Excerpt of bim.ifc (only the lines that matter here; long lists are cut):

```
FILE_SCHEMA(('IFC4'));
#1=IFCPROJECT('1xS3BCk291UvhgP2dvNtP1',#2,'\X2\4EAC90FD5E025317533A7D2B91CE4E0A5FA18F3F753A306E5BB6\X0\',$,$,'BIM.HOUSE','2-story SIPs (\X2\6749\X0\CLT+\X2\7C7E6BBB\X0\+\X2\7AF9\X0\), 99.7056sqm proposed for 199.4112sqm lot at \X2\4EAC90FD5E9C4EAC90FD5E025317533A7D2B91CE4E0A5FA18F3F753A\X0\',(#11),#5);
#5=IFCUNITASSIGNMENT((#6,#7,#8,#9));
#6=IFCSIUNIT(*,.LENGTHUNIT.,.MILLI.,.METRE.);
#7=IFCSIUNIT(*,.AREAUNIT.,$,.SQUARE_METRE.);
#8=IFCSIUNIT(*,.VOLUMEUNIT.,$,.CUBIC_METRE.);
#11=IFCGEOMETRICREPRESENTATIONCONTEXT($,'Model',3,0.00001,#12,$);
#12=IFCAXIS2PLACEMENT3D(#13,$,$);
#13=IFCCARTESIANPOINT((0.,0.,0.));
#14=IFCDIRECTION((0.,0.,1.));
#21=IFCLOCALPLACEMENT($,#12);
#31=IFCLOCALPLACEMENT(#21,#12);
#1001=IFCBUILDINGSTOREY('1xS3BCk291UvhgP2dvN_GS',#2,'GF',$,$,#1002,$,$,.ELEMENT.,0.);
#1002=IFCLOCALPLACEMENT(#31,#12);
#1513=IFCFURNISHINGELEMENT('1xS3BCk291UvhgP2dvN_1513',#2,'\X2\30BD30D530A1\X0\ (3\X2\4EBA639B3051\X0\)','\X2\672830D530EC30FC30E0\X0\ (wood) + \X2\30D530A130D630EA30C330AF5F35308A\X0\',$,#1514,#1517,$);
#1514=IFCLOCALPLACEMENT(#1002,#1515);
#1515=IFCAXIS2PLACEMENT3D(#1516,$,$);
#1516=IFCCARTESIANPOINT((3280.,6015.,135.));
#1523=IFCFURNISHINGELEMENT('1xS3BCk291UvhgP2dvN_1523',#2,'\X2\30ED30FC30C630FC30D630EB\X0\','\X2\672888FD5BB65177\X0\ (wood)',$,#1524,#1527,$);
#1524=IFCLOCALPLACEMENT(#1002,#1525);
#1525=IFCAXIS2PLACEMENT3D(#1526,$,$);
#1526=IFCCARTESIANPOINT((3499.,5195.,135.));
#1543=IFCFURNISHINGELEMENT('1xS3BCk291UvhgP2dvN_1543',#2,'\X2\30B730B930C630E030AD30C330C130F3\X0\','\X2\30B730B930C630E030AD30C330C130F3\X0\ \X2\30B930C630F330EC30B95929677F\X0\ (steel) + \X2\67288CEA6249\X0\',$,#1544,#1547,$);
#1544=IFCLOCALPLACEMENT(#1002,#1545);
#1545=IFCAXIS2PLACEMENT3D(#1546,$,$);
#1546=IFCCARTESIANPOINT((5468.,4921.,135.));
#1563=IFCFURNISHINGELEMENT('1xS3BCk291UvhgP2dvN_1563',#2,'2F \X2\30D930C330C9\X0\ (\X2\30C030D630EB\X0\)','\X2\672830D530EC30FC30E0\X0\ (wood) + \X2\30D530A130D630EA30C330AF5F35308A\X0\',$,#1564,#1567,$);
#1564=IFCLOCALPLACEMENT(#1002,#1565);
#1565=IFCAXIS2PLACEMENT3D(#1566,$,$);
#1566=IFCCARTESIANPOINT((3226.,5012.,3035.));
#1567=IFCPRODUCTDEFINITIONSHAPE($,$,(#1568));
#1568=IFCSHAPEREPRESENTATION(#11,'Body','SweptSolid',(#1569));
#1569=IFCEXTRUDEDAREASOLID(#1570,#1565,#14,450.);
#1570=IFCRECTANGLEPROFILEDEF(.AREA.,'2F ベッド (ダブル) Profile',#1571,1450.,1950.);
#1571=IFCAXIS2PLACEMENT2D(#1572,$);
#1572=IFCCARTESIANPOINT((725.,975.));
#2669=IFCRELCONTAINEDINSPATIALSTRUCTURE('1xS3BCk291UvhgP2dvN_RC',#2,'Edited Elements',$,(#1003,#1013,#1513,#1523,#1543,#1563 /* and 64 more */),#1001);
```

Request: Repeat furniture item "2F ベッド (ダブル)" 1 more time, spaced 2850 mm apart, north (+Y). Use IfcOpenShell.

```python
import numpy as np
import ifcopenshell
import ifcopenshell.api.geometry
import ifcopenshell.api.root
import ifcopenshell.util.element
import ifcopenshell.util.placement
import ifcopenshell.util.unit

model = ifcopenshell.open("bim.ifc")
unit_scale = ifcopenshell.util.unit.calculate_unit_scale(model)


def reuse_history(source, copy):
    """copy_class also copies each property set's owner history, people and application; keep the originals."""
    for rel in copy.IsDefinedBy:
        if rel.is_a("IfcRelDefinesByProperties") and (history := rel.RelatingPropertyDefinition.OwnerHistory):
            rel.RelatingPropertyDefinition.OwnerHistory = source.OwnerHistory
            ifcopenshell.util.element.remove_deep2(model, history)


source = model.by_guid("1xS3BCk291UvhgP2dvN_1563")
base = ifcopenshell.util.placement.get_local_placement(source.ObjectPlacement)
step = np.array([0.0, 1.0, 0.0]) * 2.85 / unit_scale

for i in range(1, 2):
    copy = ifcopenshell.api.root.copy_class(model, product=source)
    copy.Representation = ifcopenshell.util.element.copy_deep(
        model, source.Representation, exclude=["IfcGeometricRepresentationContext", "IfcRepresentationMap"]
    )
    reuse_history(source, copy)
    matrix = base.copy()
    matrix[:3, 3] += i * step
    print("added at", matrix[:3, 3].round(3) + 0.0)
    ifcopenshell.api.geometry.edit_object_placement(model, product=copy, matrix=matrix, is_si=False)

model.write("bim-out.ifc")
```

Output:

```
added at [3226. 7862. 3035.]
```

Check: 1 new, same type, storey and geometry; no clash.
